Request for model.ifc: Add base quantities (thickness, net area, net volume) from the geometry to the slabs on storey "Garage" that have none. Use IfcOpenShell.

First a look at what the model holds.

```python
import ifcopenshell
import ifcopenshell.util.element
import ifcopenshell.util.unit

model = ifcopenshell.open("model.ifc")
print(model.schema)
for unit_type in ("LENGTHUNIT", "AREAUNIT", "VOLUMEUNIT"):
    print(unit_type, ifcopenshell.util.unit.calculate_unit_scale(model, unit_type))
storey = next(s for s in model.by_type("IfcBuildingStorey") if s.Name == "Garage")
slabs = [e for e in ifcopenshell.util.element.get_decomposition(storey) if e.is_a("IfcSlab")]
for e in sorted(slabs, key=lambda e: e.id()):
    print(e.id(), e.is_a(), e.Name, list(ifcopenshell.util.element.get_psets(e, qtos_only=True)), sep=" | ")
```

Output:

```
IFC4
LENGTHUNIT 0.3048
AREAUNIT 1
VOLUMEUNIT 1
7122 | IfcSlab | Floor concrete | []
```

```python
import ifcopenshell
import ifcopenshell.api.pset
import ifcopenshell.geom
import ifcopenshell.util.element
import ifcopenshell.util.shape
import ifcopenshell.util.unit

model = ifcopenshell.open("model.ifc")
unit_scale = ifcopenshell.util.unit.calculate_unit_scale(model)
area_scale = ifcopenshell.util.unit.calculate_unit_scale(model, "AREAUNIT")
volume_scale = ifcopenshell.util.unit.calculate_unit_scale(model, "VOLUMEUNIT")
settings = ifcopenshell.geom.settings()

storey = next(s for s in model.by_type("IfcBuildingStorey") if s.Name == "Garage")
slabs = [e for e in ifcopenshell.util.element.get_decomposition(storey) if e.is_a("IfcSlab")]

for e in sorted(slabs, key=lambda e: e.id()):
    if ifcopenshell.util.element.get_psets(e, qtos_only=True, should_inherit=False):
        continue
    # Geometry comes back in metres, in the element's own axes.
    shape = ifcopenshell.geom.create_shape(settings, e)
    values = {
        "Width": ifcopenshell.util.shape.get_z(shape.geometry) / unit_scale,
        "NetArea": ifcopenshell.util.shape.get_footprint_area(shape.geometry) / area_scale,
        "NetVolume": ifcopenshell.util.shape.get_volume(shape.geometry) / volume_scale,
    }
    qto = ifcopenshell.api.pset.add_qto(model, product=e, name="Qto_SlabBaseQuantities")
    ifcopenshell.api.pset.edit_qto(model, qto=qto, properties=values)
    print(e.id(), {k: round(v, 3) for k, v in values.items()})

model.write("model_rev.ifc")
```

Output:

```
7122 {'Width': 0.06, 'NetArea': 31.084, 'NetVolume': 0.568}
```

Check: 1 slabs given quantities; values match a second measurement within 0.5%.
